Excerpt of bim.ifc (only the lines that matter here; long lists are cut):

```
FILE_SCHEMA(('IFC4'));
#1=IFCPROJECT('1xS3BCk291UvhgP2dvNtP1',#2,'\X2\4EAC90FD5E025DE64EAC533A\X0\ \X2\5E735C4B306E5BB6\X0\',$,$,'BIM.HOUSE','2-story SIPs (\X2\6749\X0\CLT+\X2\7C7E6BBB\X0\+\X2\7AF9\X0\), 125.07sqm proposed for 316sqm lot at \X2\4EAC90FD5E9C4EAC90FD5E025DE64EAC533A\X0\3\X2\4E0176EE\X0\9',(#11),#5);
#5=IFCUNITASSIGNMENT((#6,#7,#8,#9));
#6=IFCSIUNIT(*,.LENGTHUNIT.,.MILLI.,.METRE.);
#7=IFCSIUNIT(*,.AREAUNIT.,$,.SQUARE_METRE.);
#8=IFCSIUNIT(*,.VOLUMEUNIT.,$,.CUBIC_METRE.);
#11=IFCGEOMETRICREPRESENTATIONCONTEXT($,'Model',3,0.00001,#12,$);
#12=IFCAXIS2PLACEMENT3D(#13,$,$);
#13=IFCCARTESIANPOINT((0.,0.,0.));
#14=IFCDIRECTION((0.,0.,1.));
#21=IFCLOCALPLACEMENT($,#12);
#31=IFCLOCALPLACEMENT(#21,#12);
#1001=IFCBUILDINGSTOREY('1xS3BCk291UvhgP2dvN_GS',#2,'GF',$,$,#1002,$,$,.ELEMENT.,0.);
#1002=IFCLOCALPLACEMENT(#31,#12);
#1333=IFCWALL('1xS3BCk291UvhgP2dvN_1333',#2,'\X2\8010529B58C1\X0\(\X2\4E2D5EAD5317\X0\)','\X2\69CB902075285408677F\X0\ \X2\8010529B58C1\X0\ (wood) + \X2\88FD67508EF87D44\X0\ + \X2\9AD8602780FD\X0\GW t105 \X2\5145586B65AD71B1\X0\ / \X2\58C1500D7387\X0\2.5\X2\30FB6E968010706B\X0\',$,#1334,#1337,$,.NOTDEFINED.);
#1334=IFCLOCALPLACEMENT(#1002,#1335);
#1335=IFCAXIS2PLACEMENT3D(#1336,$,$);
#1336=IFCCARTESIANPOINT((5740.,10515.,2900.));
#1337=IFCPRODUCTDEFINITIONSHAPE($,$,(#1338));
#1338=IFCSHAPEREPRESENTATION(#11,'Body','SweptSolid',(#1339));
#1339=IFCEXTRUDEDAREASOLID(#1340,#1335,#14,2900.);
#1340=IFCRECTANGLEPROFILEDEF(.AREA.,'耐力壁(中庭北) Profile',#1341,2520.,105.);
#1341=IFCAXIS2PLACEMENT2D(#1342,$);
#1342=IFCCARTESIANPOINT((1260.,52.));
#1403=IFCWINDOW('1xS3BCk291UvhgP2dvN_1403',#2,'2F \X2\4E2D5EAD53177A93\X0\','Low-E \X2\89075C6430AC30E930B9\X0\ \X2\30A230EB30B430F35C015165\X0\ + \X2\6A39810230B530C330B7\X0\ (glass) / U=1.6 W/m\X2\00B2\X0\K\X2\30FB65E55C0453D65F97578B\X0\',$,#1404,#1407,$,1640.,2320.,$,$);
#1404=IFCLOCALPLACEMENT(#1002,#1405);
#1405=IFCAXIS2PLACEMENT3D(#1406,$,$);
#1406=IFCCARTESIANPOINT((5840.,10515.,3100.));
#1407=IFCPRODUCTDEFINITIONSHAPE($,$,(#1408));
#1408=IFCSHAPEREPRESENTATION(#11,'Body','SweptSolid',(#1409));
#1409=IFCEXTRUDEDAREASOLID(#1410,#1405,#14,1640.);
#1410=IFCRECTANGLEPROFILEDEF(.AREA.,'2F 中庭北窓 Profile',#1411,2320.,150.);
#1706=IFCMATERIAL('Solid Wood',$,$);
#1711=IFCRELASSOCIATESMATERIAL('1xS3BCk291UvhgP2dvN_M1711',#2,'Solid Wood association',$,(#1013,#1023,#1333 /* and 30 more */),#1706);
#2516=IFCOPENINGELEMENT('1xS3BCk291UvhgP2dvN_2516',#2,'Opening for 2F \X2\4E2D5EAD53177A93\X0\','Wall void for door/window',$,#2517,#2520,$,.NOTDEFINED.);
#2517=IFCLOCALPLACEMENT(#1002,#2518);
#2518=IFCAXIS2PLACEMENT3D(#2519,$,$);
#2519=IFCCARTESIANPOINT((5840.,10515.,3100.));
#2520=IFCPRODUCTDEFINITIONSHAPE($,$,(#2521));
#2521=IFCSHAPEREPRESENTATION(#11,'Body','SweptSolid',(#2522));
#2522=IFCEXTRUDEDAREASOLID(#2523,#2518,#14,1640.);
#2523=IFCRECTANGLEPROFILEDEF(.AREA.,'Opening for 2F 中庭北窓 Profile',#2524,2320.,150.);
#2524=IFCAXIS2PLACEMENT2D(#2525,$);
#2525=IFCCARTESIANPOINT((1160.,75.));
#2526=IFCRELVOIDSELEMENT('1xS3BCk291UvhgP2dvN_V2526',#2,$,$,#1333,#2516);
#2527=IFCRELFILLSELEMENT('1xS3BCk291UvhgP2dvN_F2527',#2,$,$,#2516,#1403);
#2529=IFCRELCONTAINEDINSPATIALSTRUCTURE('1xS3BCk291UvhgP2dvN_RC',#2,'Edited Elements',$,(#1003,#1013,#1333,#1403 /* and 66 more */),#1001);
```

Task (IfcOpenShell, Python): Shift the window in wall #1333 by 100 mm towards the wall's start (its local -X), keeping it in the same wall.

```python
import ifcopenshell
import ifcopenshell.api.geometry
import ifcopenshell.util.placement
import ifcopenshell.util.unit

model = ifcopenshell.open("bim.ifc")
unit_scale = ifcopenshell.util.unit.calculate_unit_scale(model)

window = model.by_guid("1xS3BCk291UvhgP2dvN_1403")
opening = window.FillsVoids[0].RelatingOpeningElement
wall = opening.VoidsElements[0].RelatingBuildingElement

wall_matrix = ifcopenshell.util.placement.get_local_placement(wall.ObjectPlacement)
shift = wall_matrix[:3, 0] * -0.1 / unit_scale
before = ifcopenshell.util.placement.get_local_placement(window.ObjectPlacement)[:3, 3].copy()

# The window is not placed relative to its opening, so move both.
for product in (opening, window):
    matrix = ifcopenshell.util.placement.get_local_placement(product.ObjectPlacement)
    matrix[:3, 3] += shift
    ifcopenshell.api.geometry.edit_object_placement(model, product=product, matrix=matrix, is_si=False)

after = ifcopenshell.util.placement.get_local_placement(window.ObjectPlacement)[:3, 3]
print("window moved by", (after - before).round(3) + 0.0)

model.write("bim_rev.ifc")
```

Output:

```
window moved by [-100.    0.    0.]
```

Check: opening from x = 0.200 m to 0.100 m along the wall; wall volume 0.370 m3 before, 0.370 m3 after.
